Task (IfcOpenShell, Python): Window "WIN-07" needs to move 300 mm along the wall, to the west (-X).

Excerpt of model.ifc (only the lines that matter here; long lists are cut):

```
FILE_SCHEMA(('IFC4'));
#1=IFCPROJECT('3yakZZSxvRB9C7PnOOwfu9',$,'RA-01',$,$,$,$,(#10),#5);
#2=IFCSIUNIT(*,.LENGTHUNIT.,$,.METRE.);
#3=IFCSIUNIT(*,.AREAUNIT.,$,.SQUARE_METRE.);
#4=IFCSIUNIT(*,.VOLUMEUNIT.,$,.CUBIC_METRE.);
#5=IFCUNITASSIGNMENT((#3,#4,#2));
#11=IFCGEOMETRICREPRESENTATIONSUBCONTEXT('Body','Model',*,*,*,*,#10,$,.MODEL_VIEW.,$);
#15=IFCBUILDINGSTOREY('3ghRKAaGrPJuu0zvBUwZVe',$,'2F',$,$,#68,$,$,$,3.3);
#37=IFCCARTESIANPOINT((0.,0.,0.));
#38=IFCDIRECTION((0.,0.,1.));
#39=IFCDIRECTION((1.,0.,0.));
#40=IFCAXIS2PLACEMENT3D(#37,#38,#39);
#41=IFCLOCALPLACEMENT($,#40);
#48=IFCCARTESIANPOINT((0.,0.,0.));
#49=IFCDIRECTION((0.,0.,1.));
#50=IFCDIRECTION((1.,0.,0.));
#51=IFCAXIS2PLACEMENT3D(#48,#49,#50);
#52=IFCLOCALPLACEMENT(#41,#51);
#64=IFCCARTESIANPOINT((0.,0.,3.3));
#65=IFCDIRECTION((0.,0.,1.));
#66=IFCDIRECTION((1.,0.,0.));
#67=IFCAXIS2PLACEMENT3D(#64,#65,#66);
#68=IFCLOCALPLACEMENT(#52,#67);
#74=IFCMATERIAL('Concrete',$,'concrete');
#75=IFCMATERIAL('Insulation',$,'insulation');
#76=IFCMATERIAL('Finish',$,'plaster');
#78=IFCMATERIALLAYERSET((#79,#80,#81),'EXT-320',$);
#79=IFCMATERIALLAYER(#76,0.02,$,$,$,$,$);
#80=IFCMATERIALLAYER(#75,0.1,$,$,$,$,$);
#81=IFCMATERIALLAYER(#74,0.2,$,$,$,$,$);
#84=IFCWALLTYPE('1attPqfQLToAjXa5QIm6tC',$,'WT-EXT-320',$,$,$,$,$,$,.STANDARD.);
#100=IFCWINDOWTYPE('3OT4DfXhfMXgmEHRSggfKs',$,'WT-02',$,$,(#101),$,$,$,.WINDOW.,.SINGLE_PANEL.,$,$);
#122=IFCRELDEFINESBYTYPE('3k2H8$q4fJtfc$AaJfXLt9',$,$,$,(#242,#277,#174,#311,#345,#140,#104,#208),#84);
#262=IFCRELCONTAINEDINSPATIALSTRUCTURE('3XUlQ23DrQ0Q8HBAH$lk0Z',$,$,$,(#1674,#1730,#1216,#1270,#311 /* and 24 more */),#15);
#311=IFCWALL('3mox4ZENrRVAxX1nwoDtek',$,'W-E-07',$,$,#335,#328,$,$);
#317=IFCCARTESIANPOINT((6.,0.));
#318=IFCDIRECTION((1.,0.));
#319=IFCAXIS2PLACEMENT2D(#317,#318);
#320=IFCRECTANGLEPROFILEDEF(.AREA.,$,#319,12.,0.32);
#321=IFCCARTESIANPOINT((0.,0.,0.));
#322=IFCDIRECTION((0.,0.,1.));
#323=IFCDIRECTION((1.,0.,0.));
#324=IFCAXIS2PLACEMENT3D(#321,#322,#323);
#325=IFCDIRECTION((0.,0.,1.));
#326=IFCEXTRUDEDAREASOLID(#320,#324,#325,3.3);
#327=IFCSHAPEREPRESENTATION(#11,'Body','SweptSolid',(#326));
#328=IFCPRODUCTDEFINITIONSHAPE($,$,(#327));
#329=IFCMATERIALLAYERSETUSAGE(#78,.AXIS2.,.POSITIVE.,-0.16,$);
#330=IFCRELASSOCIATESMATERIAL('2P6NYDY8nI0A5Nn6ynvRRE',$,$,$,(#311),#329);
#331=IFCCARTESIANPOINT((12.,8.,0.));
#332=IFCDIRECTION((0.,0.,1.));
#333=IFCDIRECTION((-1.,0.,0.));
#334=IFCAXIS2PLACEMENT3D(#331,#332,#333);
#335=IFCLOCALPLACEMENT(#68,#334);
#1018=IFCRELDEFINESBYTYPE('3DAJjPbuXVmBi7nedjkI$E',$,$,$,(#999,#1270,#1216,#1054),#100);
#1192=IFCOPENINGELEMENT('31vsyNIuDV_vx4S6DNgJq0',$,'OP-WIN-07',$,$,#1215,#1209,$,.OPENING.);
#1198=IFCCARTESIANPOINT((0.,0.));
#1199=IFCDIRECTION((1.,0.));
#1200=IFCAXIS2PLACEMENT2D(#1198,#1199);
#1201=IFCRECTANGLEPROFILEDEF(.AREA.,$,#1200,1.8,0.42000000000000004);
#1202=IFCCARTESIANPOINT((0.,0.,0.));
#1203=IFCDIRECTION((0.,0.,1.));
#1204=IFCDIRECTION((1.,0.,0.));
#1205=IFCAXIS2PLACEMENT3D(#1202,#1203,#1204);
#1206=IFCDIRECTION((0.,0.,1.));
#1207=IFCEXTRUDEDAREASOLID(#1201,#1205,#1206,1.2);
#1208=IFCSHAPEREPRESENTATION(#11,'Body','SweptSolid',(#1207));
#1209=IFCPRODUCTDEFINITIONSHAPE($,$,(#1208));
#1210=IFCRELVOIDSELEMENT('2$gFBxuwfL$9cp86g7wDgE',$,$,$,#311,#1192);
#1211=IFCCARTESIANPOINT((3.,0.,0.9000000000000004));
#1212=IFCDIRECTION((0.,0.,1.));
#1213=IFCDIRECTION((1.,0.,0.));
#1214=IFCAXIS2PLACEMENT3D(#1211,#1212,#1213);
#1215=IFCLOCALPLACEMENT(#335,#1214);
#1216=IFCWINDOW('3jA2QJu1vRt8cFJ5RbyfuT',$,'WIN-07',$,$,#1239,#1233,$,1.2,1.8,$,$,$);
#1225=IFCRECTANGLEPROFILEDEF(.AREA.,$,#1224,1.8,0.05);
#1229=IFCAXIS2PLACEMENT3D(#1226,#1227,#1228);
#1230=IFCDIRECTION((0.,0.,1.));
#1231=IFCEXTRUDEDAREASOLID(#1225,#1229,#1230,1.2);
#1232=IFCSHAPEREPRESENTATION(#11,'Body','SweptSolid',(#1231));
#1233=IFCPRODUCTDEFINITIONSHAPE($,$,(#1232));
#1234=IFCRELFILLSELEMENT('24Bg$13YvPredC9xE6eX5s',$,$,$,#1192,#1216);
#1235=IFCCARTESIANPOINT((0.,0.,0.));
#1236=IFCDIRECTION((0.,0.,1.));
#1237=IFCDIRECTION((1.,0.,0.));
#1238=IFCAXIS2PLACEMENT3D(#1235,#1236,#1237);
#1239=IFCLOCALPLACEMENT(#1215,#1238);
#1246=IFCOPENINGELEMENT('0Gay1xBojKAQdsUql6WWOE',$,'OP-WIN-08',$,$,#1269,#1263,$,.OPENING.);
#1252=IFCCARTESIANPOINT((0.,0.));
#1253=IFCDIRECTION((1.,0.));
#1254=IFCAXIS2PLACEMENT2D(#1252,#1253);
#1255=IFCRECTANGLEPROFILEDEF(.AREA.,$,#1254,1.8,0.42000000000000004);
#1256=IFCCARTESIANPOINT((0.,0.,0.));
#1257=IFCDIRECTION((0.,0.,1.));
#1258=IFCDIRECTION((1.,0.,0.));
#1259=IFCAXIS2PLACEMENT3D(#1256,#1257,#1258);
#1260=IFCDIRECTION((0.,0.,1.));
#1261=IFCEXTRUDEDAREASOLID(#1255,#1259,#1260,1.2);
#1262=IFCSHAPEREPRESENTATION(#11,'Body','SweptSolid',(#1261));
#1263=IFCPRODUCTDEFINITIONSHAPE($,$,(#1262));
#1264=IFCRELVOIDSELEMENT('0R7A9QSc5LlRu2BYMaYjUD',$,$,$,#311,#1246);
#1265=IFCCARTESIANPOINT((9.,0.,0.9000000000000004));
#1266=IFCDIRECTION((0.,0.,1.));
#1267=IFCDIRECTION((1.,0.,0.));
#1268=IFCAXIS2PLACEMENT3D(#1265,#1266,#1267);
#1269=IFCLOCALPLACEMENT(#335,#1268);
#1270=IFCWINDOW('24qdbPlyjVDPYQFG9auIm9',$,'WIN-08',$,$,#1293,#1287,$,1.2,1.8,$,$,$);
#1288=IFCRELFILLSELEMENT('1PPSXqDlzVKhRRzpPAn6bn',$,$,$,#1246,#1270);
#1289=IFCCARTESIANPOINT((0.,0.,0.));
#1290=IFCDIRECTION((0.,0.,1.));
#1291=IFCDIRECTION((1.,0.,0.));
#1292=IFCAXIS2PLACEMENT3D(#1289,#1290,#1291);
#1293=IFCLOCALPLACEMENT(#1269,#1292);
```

```python
import ifcopenshell
import ifcopenshell.api.geometry
import ifcopenshell.util.placement
import ifcopenshell.util.unit

model = ifcopenshell.open("model.ifc")
unit_scale = ifcopenshell.util.unit.calculate_unit_scale(model)

window = model.by_id(1216)
opening = window.FillsVoids[0].RelatingOpeningElement
wall = opening.VoidsElements[0].RelatingBuildingElement

wall_matrix = ifcopenshell.util.placement.get_local_placement(wall.ObjectPlacement)
shift = wall_matrix[:3, 0] * 0.3 / unit_scale
before = ifcopenshell.util.placement.get_local_placement(window.ObjectPlacement)[:3, 3].copy()

# The window is placed relative to its opening, so it follows when the opening moves.
matrix = ifcopenshell.util.placement.get_local_placement(opening.ObjectPlacement)
matrix[:3, 3] += shift
ifcopenshell.api.geometry.edit_object_placement(
    model, product=opening, matrix=matrix, is_si=False, should_transform_children=True
)

after = ifcopenshell.util.placement.get_local_placement(window.ObjectPlacement)[:3, 3]
print("window moved by", (after - before).round(3) + 0.0)

model.write("model_edited.ifc")
```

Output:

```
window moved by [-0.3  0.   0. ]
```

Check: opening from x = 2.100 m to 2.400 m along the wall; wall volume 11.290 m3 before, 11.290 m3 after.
